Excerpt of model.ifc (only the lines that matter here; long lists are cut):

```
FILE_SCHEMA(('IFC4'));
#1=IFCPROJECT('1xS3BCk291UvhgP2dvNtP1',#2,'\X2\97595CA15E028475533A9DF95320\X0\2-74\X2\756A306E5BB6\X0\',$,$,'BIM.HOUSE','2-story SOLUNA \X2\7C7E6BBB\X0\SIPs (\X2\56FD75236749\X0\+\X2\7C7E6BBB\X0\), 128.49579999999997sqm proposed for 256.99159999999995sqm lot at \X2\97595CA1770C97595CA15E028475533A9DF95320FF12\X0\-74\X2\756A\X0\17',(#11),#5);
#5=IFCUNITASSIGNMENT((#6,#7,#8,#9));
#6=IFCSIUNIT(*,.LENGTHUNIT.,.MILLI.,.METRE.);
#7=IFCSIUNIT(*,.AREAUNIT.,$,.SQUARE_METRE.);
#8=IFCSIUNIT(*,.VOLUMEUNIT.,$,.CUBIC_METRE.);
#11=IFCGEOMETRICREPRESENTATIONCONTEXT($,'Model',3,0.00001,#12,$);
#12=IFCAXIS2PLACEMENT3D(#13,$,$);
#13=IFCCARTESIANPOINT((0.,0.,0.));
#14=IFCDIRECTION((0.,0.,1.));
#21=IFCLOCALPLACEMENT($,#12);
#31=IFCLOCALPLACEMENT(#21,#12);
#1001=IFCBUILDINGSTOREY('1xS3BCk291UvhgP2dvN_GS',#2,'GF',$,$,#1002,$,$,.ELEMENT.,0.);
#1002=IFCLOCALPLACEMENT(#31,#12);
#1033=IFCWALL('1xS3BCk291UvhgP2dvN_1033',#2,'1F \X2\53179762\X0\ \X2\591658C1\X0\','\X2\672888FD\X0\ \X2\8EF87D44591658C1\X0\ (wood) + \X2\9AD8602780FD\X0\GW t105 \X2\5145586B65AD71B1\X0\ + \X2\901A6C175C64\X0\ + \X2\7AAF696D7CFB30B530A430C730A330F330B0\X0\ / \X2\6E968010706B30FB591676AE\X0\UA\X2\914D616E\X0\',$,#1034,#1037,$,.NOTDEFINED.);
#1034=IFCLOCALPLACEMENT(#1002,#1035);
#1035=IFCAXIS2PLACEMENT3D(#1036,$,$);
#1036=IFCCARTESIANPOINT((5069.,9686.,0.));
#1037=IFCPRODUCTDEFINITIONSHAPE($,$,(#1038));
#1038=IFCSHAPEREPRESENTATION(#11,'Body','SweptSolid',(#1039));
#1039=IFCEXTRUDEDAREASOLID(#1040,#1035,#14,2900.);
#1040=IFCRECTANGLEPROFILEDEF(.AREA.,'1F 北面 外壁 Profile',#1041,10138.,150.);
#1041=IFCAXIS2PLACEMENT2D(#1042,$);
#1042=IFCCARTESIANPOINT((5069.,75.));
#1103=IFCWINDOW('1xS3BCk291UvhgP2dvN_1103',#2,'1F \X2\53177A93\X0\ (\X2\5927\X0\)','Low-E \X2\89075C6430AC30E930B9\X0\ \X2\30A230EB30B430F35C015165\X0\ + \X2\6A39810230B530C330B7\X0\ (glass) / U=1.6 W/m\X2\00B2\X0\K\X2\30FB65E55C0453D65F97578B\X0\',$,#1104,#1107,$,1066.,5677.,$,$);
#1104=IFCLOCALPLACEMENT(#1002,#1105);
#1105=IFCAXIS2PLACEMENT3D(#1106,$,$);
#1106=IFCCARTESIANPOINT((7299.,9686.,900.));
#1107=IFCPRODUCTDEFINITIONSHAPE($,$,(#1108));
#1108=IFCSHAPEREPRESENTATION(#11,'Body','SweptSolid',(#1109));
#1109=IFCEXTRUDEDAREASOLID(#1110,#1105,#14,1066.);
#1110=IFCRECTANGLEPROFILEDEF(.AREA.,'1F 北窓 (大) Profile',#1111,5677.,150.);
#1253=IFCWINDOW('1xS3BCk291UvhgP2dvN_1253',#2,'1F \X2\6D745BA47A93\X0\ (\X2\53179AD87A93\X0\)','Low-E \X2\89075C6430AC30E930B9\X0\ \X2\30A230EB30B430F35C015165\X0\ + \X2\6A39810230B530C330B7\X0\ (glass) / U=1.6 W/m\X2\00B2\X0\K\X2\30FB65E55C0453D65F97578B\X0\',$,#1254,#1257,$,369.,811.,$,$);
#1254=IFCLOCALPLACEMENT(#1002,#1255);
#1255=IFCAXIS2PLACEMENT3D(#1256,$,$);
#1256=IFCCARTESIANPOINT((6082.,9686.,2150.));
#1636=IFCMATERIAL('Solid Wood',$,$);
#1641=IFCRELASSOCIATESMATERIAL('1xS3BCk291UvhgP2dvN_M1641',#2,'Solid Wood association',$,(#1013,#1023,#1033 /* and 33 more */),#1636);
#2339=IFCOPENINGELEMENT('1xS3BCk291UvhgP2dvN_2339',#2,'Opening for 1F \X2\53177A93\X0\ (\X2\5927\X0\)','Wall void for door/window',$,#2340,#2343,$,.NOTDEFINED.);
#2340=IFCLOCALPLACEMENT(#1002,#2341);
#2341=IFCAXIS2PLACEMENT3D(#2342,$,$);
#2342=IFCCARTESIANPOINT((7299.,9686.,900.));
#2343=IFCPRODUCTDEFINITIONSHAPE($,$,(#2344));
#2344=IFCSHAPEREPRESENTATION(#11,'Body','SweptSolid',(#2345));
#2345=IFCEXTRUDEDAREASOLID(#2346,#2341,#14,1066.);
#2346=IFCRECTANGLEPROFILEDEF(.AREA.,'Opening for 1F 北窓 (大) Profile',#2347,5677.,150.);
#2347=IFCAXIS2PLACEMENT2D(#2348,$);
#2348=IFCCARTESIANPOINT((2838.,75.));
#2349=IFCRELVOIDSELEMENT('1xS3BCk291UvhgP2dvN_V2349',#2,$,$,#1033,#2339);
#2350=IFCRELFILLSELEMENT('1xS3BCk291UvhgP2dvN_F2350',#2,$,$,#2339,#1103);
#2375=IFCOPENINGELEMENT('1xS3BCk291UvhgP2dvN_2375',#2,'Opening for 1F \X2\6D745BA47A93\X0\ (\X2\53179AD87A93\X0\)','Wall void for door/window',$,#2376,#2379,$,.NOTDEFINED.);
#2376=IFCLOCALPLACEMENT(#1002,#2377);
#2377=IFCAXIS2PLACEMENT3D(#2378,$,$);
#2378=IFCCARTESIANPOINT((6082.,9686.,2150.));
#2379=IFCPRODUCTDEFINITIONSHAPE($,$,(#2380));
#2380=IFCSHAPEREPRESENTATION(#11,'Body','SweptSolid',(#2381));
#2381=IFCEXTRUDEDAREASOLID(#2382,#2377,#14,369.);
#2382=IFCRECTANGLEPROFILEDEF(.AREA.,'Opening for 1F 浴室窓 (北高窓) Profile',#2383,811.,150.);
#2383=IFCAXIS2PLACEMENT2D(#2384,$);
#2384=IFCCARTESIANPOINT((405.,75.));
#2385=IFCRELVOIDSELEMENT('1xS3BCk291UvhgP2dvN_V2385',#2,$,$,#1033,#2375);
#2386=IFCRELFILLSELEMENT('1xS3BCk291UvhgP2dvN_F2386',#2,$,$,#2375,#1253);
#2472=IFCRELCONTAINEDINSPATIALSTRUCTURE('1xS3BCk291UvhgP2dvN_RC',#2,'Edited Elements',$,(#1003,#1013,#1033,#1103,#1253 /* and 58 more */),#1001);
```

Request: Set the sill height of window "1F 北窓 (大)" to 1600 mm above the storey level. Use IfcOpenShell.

```python
import numpy as np
import ifcopenshell
import ifcopenshell.api.geometry
import ifcopenshell.geom
import ifcopenshell.util.element
import ifcopenshell.util.placement
import ifcopenshell.util.shape
import ifcopenshell.util.unit

model = ifcopenshell.open("model.ifc")
unit_scale = ifcopenshell.util.unit.calculate_unit_scale(model)

window = model.by_id(1103)
opening = window.FillsVoids[0].RelatingOpeningElement
storey = ifcopenshell.util.element.get_container(window, ifc_class="IfcBuildingStorey")
level = ifcopenshell.util.placement.get_local_placement(storey.ObjectPlacement)[2, 3]

# The opening's origin need not be at the sill, so measure its lowest point.
shape = ifcopenshell.geom.create_shape(ifcopenshell.geom.settings(), opening)
bottom = ifcopenshell.util.shape.get_shape_bottom_elevation(shape, shape.geometry) / unit_scale
dz = level + 1600.0 - bottom

shift = np.array([0.0, 0.0, dz])
# The window is not placed relative to its opening, so move both.
for product in (opening, window):
    matrix = ifcopenshell.util.placement.get_local_placement(product.ObjectPlacement)
    matrix[:3, 3] += shift
    ifcopenshell.api.geometry.edit_object_placement(model, product=product, matrix=matrix, is_si=False)

print(f"moved by {dz * unit_scale:+.3f} m")

model.write("model_updated.ifc")
```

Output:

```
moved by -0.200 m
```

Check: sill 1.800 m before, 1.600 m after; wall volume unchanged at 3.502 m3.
